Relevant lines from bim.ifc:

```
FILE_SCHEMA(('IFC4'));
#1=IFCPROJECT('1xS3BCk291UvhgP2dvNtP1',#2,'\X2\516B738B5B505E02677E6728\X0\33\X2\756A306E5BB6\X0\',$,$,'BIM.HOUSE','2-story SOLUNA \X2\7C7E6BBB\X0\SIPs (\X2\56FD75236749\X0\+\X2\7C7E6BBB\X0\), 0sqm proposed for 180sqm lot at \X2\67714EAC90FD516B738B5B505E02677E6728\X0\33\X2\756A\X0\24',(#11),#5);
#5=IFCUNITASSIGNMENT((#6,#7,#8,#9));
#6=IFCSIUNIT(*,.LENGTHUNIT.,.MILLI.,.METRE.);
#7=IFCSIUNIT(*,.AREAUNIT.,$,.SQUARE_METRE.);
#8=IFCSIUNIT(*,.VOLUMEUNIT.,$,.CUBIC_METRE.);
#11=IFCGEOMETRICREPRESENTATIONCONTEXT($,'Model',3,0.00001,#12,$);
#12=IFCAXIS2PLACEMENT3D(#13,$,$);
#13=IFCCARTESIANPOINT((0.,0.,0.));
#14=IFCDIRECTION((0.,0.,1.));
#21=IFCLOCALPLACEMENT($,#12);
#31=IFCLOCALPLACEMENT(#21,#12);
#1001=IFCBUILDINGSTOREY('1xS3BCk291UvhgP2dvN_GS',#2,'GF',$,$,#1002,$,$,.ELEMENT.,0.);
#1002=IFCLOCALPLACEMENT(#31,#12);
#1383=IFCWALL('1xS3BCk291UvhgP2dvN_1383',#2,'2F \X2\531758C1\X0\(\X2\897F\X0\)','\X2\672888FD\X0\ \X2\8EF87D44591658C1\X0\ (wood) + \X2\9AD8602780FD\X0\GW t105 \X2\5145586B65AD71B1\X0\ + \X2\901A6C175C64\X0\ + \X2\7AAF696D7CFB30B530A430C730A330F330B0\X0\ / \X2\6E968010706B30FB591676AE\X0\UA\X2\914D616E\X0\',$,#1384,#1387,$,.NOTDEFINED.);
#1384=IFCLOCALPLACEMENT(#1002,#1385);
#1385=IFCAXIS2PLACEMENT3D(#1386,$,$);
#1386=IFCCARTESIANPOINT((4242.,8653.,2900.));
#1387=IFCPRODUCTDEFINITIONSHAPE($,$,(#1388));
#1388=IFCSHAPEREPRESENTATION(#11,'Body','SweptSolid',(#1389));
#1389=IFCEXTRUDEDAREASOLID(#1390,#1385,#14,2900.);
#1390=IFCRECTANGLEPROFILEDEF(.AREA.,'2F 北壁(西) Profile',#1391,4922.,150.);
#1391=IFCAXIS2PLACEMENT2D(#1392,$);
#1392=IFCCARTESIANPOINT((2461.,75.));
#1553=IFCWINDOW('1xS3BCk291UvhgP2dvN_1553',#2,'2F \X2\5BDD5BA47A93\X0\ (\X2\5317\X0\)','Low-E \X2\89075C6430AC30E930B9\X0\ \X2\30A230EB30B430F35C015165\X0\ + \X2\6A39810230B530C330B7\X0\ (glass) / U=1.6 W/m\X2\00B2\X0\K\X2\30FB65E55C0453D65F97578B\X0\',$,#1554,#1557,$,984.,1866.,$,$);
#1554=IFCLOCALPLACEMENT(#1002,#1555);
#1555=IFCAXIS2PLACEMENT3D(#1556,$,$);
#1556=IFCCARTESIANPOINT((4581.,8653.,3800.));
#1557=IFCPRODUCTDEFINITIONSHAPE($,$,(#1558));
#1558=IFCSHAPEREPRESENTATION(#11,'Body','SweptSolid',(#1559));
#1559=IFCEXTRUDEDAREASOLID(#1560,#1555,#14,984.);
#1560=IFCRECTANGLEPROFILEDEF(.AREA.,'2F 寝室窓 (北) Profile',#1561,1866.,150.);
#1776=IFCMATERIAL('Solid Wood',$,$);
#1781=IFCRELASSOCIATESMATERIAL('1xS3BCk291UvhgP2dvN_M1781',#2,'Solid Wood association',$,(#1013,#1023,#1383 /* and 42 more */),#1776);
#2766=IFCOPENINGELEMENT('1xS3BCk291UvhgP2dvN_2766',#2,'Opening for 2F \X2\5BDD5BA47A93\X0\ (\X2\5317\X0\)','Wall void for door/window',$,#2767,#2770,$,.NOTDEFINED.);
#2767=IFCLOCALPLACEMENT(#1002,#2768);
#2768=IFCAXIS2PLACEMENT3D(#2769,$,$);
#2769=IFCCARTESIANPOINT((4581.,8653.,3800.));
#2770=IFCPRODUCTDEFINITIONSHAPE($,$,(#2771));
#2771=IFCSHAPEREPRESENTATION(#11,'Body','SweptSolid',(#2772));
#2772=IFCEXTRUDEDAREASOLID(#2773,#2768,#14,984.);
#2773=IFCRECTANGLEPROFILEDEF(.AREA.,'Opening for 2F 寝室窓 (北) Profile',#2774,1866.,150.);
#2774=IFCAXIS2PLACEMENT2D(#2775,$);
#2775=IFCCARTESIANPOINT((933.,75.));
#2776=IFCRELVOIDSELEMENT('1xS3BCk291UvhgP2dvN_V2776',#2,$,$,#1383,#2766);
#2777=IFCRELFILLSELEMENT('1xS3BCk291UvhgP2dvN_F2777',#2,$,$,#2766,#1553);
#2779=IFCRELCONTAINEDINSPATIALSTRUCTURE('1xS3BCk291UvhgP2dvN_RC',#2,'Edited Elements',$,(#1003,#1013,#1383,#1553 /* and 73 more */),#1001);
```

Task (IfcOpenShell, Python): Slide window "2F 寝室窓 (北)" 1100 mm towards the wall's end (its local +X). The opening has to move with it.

```python
import ifcopenshell
import ifcopenshell.api.geometry
import ifcopenshell.util.placement
import ifcopenshell.util.unit

model = ifcopenshell.open("bim.ifc")
unit_scale = ifcopenshell.util.unit.calculate_unit_scale(model)

window = model.by_id(1553)
opening = window.FillsVoids[0].RelatingOpeningElement
wall = opening.VoidsElements[0].RelatingBuildingElement

wall_matrix = ifcopenshell.util.placement.get_local_placement(wall.ObjectPlacement)
shift = wall_matrix[:3, 0] * 1.1 / unit_scale
before = ifcopenshell.util.placement.get_local_placement(window.ObjectPlacement)[:3, 3].copy()

# The window is not placed relative to its opening, so move both.
for product in (opening, window):
    matrix = ifcopenshell.util.placement.get_local_placement(product.ObjectPlacement)
    matrix[:3, 3] += shift
    ifcopenshell.api.geometry.edit_object_placement(model, product=product, matrix=matrix, is_si=False)

after = ifcopenshell.util.placement.get_local_placement(window.ObjectPlacement)[:3, 3]
print("window moved by", (after - before).round(3) + 0.0)

model.write("bim_v2.ifc")
```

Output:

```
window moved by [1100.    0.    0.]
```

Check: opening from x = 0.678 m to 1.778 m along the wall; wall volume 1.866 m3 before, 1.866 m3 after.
